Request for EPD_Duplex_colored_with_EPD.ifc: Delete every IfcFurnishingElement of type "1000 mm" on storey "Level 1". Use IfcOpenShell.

First a look at what the model holds.

```python
import ifcopenshell
import ifcopenshell.util.element

model = ifcopenshell.open("EPD_Duplex_colored_with_EPD.ifc")
print(model.schema)
storey = next(s for s in model.by_type("IfcBuildingStorey") if s.Name == "Level 1")
furniture = [e for e in ifcopenshell.util.element.get_decomposition(storey) if e.is_a("IfcFurnishingElement")]
seen = {}
for e in furniture:
    element_type = ifcopenshell.util.element.get_type(e)
    name = element_type.Name if element_type not in (None, e) else None
    seen[name] = seen.get(name, 0) + 1
for name, count in sorted(seen.items(), key=str):
    print(count, "x", name)
```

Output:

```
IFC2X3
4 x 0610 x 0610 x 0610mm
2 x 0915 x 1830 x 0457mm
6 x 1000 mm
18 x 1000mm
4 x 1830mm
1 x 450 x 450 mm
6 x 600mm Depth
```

```python
import ifcopenshell
import ifcopenshell.api.root
import ifcopenshell.util.element

model = ifcopenshell.open("EPD_Duplex_colored_with_EPD.ifc")

storey = next(s for s in model.by_type("IfcBuildingStorey") if s.Name == "Level 1")
furniture = [e for e in ifcopenshell.util.element.get_decomposition(storey) if e.is_a("IfcFurnishingElement")]
targets = [e for e in furniture if (t := ifcopenshell.util.element.get_type(e)) not in (None, e) and t.Name == "1000 mm"]

for e in targets:
    ifcopenshell.api.root.remove_product(model, product=e)
print(len(targets), "removed")

model.write("EPD_Duplex_colored_with_EPD_edited.ifc")
```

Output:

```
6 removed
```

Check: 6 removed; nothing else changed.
